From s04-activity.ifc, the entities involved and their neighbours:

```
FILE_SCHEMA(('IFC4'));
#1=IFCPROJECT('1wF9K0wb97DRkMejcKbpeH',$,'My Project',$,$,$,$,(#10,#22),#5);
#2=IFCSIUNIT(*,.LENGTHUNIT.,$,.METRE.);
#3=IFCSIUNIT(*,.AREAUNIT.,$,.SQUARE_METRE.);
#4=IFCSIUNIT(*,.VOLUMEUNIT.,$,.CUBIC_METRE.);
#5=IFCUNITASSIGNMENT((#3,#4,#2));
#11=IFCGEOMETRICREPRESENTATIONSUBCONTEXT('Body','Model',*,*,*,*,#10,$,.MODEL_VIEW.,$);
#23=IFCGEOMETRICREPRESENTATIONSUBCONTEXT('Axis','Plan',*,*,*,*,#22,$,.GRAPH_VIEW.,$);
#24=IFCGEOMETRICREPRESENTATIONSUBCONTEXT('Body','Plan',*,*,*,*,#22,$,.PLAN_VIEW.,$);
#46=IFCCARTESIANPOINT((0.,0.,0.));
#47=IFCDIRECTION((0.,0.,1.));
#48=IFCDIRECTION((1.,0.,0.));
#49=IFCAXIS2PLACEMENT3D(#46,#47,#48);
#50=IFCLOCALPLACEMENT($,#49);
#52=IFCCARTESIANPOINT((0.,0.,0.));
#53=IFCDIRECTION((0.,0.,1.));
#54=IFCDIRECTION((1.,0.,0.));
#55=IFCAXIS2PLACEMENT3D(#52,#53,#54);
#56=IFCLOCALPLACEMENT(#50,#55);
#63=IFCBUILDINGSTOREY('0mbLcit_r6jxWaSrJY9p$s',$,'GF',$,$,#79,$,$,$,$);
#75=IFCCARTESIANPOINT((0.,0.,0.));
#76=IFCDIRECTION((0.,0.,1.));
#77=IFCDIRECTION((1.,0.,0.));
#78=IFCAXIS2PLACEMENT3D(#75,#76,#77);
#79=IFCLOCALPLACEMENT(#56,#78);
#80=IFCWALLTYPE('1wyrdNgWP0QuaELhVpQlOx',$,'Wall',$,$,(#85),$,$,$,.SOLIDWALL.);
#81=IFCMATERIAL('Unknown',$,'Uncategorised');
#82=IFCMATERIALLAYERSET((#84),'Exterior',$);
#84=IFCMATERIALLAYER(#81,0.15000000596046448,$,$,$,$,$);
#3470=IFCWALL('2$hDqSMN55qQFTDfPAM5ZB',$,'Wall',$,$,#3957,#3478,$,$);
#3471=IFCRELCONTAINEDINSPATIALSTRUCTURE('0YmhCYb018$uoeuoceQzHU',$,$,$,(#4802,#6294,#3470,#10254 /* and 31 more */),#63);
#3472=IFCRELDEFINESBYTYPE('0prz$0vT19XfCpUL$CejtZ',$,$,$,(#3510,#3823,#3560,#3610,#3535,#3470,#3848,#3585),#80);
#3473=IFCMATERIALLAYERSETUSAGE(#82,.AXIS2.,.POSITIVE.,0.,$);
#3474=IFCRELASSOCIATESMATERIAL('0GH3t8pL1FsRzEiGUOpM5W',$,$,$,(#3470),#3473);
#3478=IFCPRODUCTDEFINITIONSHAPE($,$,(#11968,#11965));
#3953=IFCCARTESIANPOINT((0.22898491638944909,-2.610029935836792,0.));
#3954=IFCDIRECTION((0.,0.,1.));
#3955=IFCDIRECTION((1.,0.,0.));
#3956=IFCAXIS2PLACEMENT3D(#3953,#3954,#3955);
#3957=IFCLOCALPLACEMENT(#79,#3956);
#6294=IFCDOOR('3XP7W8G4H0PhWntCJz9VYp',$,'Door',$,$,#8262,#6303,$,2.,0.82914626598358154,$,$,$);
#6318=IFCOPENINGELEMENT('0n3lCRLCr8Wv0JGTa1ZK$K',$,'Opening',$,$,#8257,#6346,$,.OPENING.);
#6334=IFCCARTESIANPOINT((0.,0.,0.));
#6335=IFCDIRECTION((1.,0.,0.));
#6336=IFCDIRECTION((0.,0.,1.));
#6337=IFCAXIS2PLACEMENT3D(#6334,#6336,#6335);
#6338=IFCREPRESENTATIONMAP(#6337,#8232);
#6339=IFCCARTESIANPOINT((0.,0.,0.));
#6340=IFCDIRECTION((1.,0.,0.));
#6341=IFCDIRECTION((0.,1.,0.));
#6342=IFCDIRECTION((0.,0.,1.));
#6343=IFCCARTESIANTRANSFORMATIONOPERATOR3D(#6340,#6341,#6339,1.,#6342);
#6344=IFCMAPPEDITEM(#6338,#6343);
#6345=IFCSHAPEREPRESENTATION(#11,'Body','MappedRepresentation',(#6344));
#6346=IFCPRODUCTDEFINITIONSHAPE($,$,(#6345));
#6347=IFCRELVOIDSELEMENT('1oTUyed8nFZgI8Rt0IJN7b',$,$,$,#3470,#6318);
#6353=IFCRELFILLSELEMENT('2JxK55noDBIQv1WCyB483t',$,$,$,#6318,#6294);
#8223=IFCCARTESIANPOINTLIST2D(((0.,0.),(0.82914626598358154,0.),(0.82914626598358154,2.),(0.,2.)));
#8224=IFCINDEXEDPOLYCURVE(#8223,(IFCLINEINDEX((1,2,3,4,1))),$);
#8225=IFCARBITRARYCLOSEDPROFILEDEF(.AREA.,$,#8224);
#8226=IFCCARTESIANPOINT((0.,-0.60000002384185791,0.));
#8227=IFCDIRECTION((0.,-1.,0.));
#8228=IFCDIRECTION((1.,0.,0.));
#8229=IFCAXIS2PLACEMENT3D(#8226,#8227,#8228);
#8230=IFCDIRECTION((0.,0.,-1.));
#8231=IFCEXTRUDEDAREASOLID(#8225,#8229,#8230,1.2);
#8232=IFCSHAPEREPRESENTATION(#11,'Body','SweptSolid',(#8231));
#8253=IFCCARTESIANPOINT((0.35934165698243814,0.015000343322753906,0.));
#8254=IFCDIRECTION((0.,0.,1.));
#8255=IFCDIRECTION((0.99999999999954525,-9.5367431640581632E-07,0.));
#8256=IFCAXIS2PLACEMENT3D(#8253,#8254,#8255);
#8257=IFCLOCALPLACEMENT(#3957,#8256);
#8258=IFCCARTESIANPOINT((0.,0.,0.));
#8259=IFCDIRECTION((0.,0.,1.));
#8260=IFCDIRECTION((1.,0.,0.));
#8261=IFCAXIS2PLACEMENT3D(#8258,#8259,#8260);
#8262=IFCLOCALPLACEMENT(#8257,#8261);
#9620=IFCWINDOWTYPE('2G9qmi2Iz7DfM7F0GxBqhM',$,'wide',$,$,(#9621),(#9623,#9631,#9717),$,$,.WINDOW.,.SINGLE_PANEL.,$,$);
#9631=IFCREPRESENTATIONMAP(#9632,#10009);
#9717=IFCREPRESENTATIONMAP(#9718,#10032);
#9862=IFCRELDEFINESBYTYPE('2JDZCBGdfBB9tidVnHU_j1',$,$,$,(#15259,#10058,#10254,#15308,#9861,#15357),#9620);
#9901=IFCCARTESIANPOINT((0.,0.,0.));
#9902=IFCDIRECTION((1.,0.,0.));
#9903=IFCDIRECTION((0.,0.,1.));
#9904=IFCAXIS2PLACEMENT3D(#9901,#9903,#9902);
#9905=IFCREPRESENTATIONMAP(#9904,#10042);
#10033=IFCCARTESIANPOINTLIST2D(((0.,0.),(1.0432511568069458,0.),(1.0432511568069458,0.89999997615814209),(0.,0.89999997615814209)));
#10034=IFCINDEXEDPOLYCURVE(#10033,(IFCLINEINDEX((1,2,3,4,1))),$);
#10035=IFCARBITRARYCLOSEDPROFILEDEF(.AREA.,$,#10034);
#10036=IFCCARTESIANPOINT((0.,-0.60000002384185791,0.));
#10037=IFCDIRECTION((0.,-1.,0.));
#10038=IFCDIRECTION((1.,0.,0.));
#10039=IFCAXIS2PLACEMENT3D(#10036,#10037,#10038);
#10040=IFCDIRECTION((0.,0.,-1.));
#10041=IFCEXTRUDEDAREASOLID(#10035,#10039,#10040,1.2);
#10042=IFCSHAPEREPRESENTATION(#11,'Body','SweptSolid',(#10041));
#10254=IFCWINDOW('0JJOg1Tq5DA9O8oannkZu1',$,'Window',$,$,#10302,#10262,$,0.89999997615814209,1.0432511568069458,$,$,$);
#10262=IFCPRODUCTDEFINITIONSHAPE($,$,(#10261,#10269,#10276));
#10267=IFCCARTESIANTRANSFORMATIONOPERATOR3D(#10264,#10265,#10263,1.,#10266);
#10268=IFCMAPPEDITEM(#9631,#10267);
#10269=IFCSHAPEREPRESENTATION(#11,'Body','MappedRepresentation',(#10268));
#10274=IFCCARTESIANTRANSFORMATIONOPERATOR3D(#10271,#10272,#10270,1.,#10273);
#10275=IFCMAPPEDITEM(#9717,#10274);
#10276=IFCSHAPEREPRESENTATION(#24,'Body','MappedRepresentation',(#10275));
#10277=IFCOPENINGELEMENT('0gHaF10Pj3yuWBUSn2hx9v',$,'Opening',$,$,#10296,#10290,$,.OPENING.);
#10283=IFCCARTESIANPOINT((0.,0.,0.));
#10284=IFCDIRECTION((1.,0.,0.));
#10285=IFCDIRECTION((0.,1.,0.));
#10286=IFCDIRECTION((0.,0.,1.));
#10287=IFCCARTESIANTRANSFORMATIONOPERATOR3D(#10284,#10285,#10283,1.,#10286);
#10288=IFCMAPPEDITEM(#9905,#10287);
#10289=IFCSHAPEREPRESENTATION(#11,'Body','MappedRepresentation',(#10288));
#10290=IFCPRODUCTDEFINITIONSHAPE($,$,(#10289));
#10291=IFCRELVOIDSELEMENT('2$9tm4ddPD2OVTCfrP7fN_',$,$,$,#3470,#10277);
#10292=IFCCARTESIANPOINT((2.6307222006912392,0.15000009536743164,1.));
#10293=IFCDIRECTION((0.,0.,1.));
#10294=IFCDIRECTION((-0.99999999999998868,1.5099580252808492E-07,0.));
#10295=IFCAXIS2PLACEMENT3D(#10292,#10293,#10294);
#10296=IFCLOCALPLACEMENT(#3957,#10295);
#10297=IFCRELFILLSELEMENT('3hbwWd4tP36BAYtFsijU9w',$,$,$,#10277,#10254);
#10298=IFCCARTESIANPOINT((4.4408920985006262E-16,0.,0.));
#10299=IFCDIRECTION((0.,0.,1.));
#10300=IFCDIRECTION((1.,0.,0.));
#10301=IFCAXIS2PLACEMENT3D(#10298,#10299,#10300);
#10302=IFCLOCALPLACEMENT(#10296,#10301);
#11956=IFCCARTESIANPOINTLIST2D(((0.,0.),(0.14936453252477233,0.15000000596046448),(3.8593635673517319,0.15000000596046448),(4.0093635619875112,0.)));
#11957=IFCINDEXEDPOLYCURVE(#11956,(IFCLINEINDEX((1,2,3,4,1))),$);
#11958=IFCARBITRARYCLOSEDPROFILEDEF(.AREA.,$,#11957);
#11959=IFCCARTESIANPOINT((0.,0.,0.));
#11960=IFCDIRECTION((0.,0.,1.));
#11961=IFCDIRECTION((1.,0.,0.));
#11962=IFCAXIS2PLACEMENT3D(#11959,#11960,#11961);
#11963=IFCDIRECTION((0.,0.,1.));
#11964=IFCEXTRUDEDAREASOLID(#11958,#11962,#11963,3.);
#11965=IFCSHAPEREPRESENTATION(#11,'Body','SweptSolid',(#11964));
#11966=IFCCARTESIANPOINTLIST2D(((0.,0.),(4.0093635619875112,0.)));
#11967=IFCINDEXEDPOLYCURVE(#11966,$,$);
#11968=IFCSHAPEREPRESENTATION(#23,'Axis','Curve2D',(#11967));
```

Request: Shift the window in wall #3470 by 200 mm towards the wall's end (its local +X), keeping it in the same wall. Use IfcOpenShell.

```python
import ifcopenshell
import ifcopenshell.api.geometry
import ifcopenshell.util.placement

model = ifcopenshell.open("s04-activity.ifc")

window = model.by_id(10254)
opening = window.FillsVoids[0].RelatingOpeningElement
wall = opening.VoidsElements[0].RelatingBuildingElement

wall_matrix = ifcopenshell.util.placement.get_local_placement(wall.ObjectPlacement)
shift = wall_matrix[:3, 0] * 0.2
before = ifcopenshell.util.placement.get_local_placement(window.ObjectPlacement)[:3, 3].copy()

# The window is placed relative to its opening, so it follows when the opening moves.
matrix = ifcopenshell.util.placement.get_local_placement(opening.ObjectPlacement)
matrix[:3, 3] += shift
ifcopenshell.api.geometry.edit_object_placement(
    model, product=opening, matrix=matrix, is_si=False, should_transform_children=True
)

after = ifcopenshell.util.placement.get_local_placement(window.ObjectPlacement)[:3, 3]
print("window moved by", (after - before).round(3) + 0.0)

model.write("s04-activity_updated.ifc")
```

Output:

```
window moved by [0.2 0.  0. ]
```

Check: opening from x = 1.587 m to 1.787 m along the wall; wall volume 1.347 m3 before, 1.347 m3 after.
